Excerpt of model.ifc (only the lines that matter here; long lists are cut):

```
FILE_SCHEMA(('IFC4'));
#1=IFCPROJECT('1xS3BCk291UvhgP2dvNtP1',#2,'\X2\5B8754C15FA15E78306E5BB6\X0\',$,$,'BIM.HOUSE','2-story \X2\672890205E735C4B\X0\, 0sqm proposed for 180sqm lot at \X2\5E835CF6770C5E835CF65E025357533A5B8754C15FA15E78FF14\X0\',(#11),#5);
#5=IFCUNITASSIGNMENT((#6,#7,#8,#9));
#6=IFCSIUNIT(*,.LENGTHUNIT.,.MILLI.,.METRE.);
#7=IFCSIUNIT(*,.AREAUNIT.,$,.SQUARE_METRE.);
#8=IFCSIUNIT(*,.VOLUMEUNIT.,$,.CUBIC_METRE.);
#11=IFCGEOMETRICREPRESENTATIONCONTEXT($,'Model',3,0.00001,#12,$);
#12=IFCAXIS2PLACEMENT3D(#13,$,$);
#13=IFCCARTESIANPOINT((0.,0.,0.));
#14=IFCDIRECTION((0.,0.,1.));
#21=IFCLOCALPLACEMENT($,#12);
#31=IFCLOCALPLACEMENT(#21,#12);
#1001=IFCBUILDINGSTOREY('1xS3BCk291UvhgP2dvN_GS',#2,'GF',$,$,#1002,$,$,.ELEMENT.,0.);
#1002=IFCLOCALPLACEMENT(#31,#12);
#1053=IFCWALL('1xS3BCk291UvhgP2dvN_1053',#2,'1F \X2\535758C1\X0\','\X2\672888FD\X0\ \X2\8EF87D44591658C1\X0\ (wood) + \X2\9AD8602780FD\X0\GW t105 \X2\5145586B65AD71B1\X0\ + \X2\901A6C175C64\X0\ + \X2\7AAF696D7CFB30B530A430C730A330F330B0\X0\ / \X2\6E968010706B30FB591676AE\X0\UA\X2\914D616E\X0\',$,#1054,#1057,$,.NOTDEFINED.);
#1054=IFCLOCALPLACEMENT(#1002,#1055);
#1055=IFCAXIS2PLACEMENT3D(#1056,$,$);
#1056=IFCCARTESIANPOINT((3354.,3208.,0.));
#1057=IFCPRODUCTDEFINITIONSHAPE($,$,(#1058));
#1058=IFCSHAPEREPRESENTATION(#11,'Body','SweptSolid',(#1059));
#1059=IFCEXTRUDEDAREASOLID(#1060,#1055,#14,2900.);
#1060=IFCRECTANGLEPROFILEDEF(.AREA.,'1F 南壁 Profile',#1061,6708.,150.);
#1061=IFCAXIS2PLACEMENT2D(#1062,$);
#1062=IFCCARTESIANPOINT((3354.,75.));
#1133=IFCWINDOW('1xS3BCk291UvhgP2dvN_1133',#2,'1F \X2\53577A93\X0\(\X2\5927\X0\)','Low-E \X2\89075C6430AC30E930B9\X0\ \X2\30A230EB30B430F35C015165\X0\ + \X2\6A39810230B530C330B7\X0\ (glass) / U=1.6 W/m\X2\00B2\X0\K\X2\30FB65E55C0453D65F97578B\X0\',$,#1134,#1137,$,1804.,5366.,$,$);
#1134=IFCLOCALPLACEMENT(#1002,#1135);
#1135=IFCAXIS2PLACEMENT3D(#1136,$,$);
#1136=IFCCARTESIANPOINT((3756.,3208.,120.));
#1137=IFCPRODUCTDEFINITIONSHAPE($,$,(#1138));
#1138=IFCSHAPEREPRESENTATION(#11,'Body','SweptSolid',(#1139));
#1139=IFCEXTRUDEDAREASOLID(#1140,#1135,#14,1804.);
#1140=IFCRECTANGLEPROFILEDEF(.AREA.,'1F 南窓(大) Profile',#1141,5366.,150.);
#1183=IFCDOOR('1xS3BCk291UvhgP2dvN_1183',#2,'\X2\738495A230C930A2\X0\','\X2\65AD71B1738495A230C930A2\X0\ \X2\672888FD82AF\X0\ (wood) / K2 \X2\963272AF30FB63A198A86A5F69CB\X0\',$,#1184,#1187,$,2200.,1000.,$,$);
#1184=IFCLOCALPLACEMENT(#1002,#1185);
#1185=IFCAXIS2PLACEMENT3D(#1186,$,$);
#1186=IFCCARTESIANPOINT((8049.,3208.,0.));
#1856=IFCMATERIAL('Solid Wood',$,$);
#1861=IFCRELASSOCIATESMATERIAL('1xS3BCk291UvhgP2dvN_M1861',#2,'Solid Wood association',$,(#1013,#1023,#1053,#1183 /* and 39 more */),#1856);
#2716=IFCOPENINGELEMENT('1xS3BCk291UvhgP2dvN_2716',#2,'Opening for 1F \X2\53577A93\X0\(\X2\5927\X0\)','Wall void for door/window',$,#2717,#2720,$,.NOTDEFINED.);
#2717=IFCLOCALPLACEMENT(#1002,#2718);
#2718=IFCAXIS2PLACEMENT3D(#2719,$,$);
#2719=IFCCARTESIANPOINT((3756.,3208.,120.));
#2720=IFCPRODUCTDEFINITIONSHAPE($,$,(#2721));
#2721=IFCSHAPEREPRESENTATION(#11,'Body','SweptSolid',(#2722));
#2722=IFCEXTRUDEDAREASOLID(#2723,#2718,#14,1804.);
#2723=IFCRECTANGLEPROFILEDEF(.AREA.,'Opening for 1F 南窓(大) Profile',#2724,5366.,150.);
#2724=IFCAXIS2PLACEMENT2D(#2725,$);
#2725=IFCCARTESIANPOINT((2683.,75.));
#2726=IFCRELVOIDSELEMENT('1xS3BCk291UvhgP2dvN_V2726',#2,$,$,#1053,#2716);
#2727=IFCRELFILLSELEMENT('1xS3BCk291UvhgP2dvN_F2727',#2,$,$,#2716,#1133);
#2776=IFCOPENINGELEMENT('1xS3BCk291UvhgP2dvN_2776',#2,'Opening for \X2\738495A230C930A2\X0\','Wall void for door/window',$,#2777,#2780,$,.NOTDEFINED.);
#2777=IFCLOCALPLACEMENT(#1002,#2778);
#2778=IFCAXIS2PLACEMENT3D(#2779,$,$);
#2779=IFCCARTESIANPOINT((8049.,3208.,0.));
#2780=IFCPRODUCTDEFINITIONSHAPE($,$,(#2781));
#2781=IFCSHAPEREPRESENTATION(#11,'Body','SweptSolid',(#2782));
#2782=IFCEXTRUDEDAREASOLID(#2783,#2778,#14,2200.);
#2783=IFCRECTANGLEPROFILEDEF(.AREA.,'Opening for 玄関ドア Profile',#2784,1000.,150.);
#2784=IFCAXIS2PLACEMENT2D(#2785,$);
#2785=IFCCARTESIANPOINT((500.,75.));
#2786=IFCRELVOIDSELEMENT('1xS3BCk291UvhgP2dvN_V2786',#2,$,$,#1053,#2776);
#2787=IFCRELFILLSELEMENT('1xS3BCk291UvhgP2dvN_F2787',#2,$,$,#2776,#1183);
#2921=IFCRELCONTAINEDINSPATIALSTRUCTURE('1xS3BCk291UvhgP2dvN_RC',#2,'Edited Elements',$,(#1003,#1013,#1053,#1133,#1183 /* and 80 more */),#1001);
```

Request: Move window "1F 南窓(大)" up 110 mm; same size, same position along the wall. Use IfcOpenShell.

```python
import numpy as np
import ifcopenshell
import ifcopenshell.api.geometry
import ifcopenshell.util.placement
import ifcopenshell.util.unit

model = ifcopenshell.open("model.ifc")
unit_scale = ifcopenshell.util.unit.calculate_unit_scale(model)

window = model.by_guid("1xS3BCk291UvhgP2dvN_1133")
opening = window.FillsVoids[0].RelatingOpeningElement
dz = 110.0

shift = np.array([0.0, 0.0, dz])
# The window is not placed relative to its opening, so move both.
for product in (opening, window):
    matrix = ifcopenshell.util.placement.get_local_placement(product.ObjectPlacement)
    matrix[:3, 3] += shift
    ifcopenshell.api.geometry.edit_object_placement(model, product=product, matrix=matrix, is_si=False)

print(f"moved by {dz * unit_scale:+.3f} m")

model.write("model_v2.ifc")
```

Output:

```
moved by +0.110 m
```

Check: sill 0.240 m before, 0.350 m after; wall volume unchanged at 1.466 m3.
